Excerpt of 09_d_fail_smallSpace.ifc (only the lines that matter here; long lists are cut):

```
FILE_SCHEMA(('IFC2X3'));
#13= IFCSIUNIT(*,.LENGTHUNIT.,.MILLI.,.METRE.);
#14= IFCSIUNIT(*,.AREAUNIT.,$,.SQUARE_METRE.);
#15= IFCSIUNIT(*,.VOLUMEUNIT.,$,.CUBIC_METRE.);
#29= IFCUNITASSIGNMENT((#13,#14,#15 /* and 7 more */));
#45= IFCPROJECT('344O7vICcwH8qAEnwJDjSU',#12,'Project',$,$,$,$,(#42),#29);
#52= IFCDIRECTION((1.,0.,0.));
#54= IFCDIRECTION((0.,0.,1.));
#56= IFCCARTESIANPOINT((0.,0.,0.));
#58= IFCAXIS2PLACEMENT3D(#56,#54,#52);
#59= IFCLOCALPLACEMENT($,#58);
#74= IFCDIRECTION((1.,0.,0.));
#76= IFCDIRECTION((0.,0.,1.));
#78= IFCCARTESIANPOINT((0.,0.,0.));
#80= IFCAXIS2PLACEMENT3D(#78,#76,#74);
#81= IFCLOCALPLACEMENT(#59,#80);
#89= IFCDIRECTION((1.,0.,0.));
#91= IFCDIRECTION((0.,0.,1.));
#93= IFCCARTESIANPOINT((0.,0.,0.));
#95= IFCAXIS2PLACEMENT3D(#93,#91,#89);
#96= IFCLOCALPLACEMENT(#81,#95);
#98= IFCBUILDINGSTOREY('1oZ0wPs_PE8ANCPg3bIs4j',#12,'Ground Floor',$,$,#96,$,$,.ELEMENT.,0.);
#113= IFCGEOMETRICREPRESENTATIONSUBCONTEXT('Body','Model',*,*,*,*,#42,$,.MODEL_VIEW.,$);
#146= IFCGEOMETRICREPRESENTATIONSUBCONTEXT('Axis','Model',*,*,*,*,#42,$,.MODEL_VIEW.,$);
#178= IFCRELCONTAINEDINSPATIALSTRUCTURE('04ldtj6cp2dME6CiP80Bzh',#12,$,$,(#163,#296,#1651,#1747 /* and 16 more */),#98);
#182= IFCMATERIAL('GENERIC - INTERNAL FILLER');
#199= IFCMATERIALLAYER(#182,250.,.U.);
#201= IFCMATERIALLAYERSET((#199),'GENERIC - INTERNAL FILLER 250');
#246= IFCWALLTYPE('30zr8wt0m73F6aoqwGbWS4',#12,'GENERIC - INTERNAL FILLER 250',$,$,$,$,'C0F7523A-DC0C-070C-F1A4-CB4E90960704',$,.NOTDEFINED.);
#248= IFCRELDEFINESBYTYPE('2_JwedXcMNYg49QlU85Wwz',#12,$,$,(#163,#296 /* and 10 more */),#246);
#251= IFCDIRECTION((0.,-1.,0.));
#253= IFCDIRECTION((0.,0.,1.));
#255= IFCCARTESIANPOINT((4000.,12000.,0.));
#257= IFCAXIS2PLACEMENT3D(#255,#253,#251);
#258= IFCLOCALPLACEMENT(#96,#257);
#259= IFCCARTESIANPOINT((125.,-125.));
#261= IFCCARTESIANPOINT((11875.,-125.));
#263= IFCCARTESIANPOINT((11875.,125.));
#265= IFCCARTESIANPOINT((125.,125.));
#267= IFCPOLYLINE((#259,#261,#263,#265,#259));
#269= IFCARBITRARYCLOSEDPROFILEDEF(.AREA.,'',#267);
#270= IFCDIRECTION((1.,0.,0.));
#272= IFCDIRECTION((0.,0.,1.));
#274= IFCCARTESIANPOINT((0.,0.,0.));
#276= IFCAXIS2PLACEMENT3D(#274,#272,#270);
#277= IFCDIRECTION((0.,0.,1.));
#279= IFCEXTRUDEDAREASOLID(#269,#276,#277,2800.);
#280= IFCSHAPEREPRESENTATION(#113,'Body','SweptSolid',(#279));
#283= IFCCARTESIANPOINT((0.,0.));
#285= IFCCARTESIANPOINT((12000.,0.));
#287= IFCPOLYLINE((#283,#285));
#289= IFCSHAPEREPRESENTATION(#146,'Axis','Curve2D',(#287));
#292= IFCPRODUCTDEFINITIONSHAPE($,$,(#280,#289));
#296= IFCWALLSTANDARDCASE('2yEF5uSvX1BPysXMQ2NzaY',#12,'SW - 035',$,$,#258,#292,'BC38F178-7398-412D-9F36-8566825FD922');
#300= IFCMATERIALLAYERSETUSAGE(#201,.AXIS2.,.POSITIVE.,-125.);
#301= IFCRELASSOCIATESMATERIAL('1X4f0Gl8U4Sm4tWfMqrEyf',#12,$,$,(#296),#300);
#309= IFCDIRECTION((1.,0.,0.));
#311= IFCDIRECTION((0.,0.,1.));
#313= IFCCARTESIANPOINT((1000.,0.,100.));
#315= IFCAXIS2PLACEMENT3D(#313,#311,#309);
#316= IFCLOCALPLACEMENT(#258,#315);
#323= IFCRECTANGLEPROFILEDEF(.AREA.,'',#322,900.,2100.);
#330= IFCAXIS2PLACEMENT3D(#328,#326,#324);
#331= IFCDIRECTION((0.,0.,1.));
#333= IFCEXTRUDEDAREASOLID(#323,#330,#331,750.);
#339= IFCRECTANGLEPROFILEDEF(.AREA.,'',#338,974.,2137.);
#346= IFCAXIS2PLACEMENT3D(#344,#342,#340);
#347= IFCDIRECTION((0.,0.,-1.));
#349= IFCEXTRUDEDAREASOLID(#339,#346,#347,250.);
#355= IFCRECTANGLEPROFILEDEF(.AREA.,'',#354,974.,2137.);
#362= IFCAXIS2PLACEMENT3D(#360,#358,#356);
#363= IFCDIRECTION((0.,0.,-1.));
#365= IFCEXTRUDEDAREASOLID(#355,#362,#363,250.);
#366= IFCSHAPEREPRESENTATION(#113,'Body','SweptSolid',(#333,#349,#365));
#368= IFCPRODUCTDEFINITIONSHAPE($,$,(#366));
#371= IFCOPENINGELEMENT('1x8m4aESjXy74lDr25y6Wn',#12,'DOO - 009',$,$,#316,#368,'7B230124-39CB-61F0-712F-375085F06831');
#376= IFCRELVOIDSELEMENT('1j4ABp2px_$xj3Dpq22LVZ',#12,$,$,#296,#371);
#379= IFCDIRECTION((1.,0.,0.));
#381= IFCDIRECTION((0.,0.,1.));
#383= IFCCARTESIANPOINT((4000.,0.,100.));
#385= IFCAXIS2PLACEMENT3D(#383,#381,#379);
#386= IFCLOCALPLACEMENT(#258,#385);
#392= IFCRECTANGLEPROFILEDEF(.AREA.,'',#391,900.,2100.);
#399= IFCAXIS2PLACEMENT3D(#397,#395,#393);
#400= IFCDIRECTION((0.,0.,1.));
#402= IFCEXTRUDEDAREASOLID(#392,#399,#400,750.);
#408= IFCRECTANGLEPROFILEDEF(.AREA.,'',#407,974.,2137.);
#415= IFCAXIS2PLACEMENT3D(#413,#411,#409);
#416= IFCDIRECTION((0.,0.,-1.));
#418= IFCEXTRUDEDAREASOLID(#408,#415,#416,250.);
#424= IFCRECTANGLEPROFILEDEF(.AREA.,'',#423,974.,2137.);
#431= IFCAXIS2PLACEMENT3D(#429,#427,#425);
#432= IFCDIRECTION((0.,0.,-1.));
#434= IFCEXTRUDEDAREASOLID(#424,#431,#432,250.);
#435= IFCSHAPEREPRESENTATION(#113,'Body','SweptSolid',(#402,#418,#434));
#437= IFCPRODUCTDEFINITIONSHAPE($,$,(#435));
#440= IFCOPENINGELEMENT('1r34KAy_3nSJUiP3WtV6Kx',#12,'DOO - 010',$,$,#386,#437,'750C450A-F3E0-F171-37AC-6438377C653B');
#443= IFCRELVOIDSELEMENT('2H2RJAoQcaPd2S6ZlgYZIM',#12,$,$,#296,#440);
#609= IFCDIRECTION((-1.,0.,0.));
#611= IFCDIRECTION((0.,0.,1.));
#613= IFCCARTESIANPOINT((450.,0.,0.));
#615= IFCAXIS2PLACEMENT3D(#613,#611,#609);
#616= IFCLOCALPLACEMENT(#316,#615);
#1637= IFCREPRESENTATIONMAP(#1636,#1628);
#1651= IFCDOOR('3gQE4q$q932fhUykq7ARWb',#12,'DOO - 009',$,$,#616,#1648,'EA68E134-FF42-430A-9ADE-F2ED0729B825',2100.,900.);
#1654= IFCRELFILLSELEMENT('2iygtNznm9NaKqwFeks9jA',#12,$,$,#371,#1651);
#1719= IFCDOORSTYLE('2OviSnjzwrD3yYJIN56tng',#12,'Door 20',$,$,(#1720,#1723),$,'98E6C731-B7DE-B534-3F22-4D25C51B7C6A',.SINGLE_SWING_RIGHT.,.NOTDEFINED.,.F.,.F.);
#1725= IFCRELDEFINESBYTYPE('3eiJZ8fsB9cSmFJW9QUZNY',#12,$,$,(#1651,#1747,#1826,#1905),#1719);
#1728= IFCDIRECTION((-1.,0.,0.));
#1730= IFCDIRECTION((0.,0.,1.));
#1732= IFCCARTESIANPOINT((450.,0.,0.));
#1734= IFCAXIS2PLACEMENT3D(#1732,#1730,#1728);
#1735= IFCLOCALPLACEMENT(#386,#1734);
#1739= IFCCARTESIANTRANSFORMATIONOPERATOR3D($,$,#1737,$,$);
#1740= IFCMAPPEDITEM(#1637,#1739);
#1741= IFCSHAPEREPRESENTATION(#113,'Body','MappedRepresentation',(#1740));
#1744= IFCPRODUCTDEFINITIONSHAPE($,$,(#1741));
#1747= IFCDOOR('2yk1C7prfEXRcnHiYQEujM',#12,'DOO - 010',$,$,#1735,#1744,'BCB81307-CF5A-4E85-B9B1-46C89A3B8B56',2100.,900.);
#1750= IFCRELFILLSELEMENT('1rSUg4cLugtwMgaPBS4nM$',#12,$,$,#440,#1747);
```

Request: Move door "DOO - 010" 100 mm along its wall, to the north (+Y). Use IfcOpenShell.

```python
import ifcopenshell
import ifcopenshell.api.geometry
import ifcopenshell.util.placement
import ifcopenshell.util.unit

model = ifcopenshell.open("09_d_fail_smallSpace.ifc")
unit_scale = ifcopenshell.util.unit.calculate_unit_scale(model)

door = model.by_guid("2yk1C7prfEXRcnHiYQEujM")
opening = door.FillsVoids[0].RelatingOpeningElement
wall = opening.VoidsElements[0].RelatingBuildingElement

wall_matrix = ifcopenshell.util.placement.get_local_placement(wall.ObjectPlacement)
shift = wall_matrix[:3, 0] * -0.1 / unit_scale
before = ifcopenshell.util.placement.get_local_placement(door.ObjectPlacement)[:3, 3].copy()

# The door is placed relative to its opening, so it follows when the opening moves.
matrix = ifcopenshell.util.placement.get_local_placement(opening.ObjectPlacement)
matrix[:3, 3] += shift
ifcopenshell.api.geometry.edit_object_placement(
    model, product=opening, matrix=matrix, is_si=False, should_transform_children=True
)

after = ifcopenshell.util.placement.get_local_placement(door.ObjectPlacement)[:3, 3]
print("door moved by", (after - before).round(3) + 0.0)

model.write("09_d_fail_smallSpace_rev.ifc")
```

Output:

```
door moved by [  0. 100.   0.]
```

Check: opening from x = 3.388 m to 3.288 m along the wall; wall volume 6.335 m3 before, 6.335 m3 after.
